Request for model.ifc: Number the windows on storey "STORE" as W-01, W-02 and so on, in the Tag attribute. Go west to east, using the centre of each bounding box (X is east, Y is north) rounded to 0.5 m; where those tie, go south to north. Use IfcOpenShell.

First a look at what the model holds.

```python
import ifcopenshell
import ifcopenshell.util.element
import ifcopenshell.util.placement

model = ifcopenshell.open("model.ifc")
print(model.schema)
storey = next(s for s in model.by_type("IfcBuildingStorey") if s.Name == "STORE")
windows = [e for e in ifcopenshell.util.element.get_decomposition(storey) if e.is_a("IfcWindow")]
for e in sorted(windows, key=lambda e: e.id()):
    origin = ifcopenshell.util.placement.get_local_placement(e.ObjectPlacement)[:3, 3]
    print(e.id(), e.Tag, e.Name, origin.round(2) + 0.0, sep=" | ")
```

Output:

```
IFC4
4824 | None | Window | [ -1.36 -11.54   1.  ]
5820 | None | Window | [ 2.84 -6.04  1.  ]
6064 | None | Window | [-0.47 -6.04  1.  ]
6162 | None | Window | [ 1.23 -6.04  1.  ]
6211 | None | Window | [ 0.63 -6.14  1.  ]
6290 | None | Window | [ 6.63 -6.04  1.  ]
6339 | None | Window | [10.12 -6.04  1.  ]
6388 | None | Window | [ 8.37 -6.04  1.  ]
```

```python
import ifcopenshell
import ifcopenshell.geom
import ifcopenshell.util.element
import ifcopenshell.util.shape

model = ifcopenshell.open("model.ifc")
settings = ifcopenshell.geom.settings()
settings.set("use-world-coords", True)


def centre(element):
    shape = ifcopenshell.geom.create_shape(settings, element)
    return ifcopenshell.util.shape.get_bbox_centroid(shape.geometry)


storey = next(s for s in model.by_type("IfcBuildingStorey") if s.Name == "STORE")
windows = [e for e in ifcopenshell.util.element.get_decomposition(storey) if e.is_a("IfcWindow")]

# Insertion points can sit at a corner or the storey origin, so sort by the geometry (in metres).
centres = {e: centre(e) for e in windows}
windows.sort(key=lambda e: (round(centres[e][0] / 0.5), centres[e][1]))

for i, e in enumerate(windows, start=1):
    number = f"W-{i:02d}"
    e.Tag = number
    print(e.id(), number)

model.write("model_updated.ifc")
```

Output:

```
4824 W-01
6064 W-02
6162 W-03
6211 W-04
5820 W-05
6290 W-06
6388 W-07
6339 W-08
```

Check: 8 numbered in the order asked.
